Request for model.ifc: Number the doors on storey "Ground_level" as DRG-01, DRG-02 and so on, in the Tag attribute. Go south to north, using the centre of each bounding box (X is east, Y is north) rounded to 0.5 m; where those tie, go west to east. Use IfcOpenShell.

First a look at what the model holds.

```python
import ifcopenshell
import ifcopenshell.util.element
import ifcopenshell.util.placement

model = ifcopenshell.open("model.ifc")
print(model.schema)
storey = next(s for s in model.by_type("IfcBuildingStorey") if s.Name == "Ground_level")
doors = [e for e in ifcopenshell.util.element.get_decomposition(storey) if e.is_a("IfcDoor")]
for e in sorted(doors, key=lambda e: e.id()):
    origin = ifcopenshell.util.placement.get_local_placement(e.ObjectPlacement)[:3, 3]
    print(e.id(), e.Tag, e.Name, origin.round(2) + 0.0, sep=" | ")
```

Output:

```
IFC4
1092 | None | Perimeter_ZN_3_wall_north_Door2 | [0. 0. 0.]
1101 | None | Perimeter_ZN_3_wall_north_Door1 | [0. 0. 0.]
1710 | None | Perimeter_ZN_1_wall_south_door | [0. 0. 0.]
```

```python
import ifcopenshell
import ifcopenshell.geom
import ifcopenshell.util.element
import ifcopenshell.util.shape

model = ifcopenshell.open("model.ifc")
settings = ifcopenshell.geom.settings()
settings.set("use-world-coords", True)


def centre(element):
    shape = ifcopenshell.geom.create_shape(settings, element)
    return ifcopenshell.util.shape.get_bbox_centroid(shape.geometry)


storey = next(s for s in model.by_type("IfcBuildingStorey") if s.Name == "Ground_level")
doors = [e for e in ifcopenshell.util.element.get_decomposition(storey) if e.is_a("IfcDoor")]

# Insertion points can sit at a corner or the storey origin, so sort by the geometry (in metres).
centres = {e: centre(e) for e in doors}
doors.sort(key=lambda e: (round(centres[e][1] / 0.5), centres[e][0]))

for i, e in enumerate(doors, start=1):
    number = f"DRG-{i:02d}"
    e.Tag = number
    print(e.id(), number)

model.write("model_v2.ifc")
```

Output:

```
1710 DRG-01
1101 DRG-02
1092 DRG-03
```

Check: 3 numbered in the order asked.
